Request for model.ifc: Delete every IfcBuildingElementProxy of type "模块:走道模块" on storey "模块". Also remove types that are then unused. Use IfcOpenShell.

First a look at what the model holds.

```python
import ifcopenshell
import ifcopenshell.util.element

model = ifcopenshell.open("model.ifc")
print(model.schema)
storey = next(s for s in model.by_type("IfcBuildingStorey") if s.Name == "模块")
proxies = [e for e in ifcopenshell.util.element.get_decomposition(storey) if e.is_a("IfcBuildingElementProxy")]
seen = {}
for e in proxies:
    element_type = ifcopenshell.util.element.get_type(e)
    name = element_type.Name if element_type not in (None, e) else None
    seen[name] = seen.get(name, 0) + 1
for name, count in sorted(seen.items(), key=str):
    print(count, "x", name)
```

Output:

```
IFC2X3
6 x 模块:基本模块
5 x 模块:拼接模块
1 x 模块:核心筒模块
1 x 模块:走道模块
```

```python
import ifcopenshell
import ifcopenshell.api.root
import ifcopenshell.util.element

model = ifcopenshell.open("model.ifc")

storey = next(s for s in model.by_type("IfcBuildingStorey") if s.Name == "模块")
proxies = [e for e in ifcopenshell.util.element.get_decomposition(storey) if e.is_a("IfcBuildingElementProxy")]
targets = [e for e in proxies if (t := ifcopenshell.util.element.get_type(e)) not in (None, e) and t.Name == "模块:走道模块"]
types = {ifcopenshell.util.element.get_type(e) for e in targets} - {None, *targets}

for e in targets:
    ifcopenshell.api.root.remove_product(model, product=e)
print(len(targets), "removed")

unused = [t for t in types if not ifcopenshell.util.element.get_types(t)]
for t in unused:
    ifcopenshell.api.root.remove_product(model, product=t)
print(len(unused), "unused types removed")

model.write("model-out.ifc")
```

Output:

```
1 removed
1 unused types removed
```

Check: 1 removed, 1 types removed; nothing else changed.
